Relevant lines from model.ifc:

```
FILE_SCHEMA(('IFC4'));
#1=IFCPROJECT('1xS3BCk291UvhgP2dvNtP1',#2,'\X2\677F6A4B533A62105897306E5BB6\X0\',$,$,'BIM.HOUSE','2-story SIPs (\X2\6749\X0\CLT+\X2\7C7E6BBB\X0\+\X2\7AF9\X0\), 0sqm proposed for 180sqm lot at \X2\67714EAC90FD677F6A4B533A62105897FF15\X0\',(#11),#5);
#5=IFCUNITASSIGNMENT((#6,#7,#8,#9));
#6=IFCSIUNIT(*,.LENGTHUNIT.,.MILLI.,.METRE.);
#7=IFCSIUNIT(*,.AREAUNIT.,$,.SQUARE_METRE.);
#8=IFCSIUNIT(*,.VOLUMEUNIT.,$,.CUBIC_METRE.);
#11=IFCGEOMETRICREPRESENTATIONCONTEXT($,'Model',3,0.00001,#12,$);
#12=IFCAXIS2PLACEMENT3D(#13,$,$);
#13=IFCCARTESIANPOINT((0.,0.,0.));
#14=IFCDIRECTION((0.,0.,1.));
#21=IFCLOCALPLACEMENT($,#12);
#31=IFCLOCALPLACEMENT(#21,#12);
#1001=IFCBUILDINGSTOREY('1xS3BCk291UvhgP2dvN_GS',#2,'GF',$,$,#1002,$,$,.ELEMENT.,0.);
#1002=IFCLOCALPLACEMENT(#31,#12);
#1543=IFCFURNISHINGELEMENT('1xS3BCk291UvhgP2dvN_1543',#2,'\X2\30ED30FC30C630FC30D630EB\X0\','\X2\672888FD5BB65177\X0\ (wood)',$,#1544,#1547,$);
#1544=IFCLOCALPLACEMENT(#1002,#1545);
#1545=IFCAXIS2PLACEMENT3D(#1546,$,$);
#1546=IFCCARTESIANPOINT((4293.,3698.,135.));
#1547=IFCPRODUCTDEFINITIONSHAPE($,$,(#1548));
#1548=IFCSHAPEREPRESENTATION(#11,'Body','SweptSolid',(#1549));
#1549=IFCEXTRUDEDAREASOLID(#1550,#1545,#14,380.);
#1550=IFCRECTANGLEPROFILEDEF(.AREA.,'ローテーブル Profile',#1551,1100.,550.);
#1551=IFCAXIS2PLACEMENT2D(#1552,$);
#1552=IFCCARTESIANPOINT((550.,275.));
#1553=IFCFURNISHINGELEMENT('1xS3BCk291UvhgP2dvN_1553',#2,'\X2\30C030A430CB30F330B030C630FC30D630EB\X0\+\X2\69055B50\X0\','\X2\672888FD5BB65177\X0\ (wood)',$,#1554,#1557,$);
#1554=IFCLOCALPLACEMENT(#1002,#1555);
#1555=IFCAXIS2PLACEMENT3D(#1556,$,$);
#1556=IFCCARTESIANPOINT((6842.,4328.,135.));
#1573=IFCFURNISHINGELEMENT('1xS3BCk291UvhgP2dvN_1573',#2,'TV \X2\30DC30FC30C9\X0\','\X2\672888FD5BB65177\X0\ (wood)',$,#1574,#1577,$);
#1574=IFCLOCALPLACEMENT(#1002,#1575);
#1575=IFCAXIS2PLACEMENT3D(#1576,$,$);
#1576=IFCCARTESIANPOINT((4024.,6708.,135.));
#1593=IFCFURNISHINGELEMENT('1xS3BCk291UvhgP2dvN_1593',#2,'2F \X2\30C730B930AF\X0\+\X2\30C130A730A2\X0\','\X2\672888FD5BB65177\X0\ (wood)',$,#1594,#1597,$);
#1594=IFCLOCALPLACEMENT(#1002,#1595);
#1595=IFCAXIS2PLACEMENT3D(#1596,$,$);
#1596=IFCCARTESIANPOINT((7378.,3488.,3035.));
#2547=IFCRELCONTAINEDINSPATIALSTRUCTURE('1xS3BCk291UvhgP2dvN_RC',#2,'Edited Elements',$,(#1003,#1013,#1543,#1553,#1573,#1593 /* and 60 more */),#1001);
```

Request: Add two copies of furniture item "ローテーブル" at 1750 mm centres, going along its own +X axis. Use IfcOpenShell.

```python
import ifcopenshell
import ifcopenshell.api.geometry
import ifcopenshell.api.root
import ifcopenshell.util.element
import ifcopenshell.util.placement
import ifcopenshell.util.unit

model = ifcopenshell.open("model.ifc")
unit_scale = ifcopenshell.util.unit.calculate_unit_scale(model)


def reuse_history(source, copy):
    """copy_class also copies each property set's owner history, people and application; keep the originals."""
    for rel in copy.IsDefinedBy:
        if rel.is_a("IfcRelDefinesByProperties") and (history := rel.RelatingPropertyDefinition.OwnerHistory):
            rel.RelatingPropertyDefinition.OwnerHistory = source.OwnerHistory
            ifcopenshell.util.element.remove_deep2(model, history)


source = model.by_guid("1xS3BCk291UvhgP2dvN_1543")
base = ifcopenshell.util.placement.get_local_placement(source.ObjectPlacement)
step = base[:3, 0] * 1.75 / unit_scale

for i in range(1, 3):
    copy = ifcopenshell.api.root.copy_class(model, product=source)
    copy.Representation = ifcopenshell.util.element.copy_deep(
        model, source.Representation, exclude=["IfcGeometricRepresentationContext", "IfcRepresentationMap"]
    )
    reuse_history(source, copy)
    matrix = base.copy()
    matrix[:3, 3] += i * step
    print("added at", matrix[:3, 3].round(3) + 0.0)
    ifcopenshell.api.geometry.edit_object_placement(model, product=copy, matrix=matrix, is_si=False)

model.write("model_rev.ifc")
```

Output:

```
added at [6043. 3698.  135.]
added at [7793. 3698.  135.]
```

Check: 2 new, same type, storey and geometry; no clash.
